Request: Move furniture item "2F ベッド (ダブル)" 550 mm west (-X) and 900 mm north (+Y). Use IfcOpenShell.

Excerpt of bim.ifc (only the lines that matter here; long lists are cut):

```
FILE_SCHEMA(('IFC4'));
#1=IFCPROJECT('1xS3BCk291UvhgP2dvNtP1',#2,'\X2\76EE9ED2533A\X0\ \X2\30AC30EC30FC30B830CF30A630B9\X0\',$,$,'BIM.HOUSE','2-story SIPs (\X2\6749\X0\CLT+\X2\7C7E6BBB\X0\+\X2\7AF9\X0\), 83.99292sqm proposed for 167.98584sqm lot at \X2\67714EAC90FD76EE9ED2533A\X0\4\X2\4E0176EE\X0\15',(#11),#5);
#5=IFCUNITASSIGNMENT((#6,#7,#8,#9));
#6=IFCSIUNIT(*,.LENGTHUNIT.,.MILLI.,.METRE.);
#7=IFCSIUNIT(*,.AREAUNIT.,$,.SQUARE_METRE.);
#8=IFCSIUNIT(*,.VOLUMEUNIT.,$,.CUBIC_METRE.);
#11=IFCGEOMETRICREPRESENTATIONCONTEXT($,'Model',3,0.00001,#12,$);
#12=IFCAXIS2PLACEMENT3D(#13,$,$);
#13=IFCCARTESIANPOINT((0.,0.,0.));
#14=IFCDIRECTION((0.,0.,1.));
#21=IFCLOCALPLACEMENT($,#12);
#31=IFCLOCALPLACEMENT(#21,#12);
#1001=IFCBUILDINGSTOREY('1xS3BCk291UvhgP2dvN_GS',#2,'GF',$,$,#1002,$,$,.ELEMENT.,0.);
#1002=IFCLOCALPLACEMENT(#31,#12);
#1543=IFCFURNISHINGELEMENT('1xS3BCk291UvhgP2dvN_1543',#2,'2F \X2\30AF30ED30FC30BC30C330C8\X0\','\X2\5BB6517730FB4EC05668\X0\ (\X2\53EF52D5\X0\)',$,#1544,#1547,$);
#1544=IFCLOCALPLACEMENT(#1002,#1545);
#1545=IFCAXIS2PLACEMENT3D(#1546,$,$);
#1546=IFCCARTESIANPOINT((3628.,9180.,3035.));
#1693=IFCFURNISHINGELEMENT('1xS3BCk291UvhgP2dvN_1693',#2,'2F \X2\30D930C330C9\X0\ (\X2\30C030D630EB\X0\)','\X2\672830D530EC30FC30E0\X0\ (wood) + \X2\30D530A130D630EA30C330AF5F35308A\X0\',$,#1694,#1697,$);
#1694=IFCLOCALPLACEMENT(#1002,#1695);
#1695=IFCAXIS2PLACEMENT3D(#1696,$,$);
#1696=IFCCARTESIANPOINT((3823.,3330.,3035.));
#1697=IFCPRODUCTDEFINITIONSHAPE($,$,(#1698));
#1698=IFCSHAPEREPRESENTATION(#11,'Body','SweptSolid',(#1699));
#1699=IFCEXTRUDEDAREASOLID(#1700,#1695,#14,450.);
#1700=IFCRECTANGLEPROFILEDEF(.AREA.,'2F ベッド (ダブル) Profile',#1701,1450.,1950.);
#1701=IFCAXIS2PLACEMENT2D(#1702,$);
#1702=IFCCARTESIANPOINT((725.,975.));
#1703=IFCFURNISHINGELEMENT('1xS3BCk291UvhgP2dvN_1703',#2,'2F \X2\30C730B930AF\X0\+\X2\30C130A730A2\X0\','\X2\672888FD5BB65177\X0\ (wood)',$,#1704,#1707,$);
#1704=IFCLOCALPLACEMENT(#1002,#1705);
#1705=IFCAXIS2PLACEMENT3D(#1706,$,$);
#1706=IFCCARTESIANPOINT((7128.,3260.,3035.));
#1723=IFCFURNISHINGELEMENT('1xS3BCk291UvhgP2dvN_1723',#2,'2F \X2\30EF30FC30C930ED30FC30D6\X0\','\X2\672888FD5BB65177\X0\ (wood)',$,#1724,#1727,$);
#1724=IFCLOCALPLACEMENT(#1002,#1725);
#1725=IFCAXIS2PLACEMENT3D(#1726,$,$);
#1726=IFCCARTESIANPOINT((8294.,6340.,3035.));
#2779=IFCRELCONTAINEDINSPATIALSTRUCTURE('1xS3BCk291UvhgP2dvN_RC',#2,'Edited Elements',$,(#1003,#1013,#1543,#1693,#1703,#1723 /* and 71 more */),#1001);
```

```python
import ifcopenshell
import ifcopenshell.api.geometry
import ifcopenshell.util.placement
import ifcopenshell.util.unit

model = ifcopenshell.open("bim.ifc")
unit_scale = ifcopenshell.util.unit.calculate_unit_scale(model)

item = model.by_guid("1xS3BCk291UvhgP2dvN_1693")
matrix = ifcopenshell.util.placement.get_local_placement(item.ObjectPlacement)
matrix[0, 3] -= 0.55 / unit_scale
matrix[1, 3] += 0.9 / unit_scale
ifcopenshell.api.geometry.edit_object_placement(model, product=item, matrix=matrix, is_si=False)

print(ifcopenshell.util.placement.get_local_placement(item.ObjectPlacement).round(3) + 0.0)

model.write("bim_updated.ifc")
```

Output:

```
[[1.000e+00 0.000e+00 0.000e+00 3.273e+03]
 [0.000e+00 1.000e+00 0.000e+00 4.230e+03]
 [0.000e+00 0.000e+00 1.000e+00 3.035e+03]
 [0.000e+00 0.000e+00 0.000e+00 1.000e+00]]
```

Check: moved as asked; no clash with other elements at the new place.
